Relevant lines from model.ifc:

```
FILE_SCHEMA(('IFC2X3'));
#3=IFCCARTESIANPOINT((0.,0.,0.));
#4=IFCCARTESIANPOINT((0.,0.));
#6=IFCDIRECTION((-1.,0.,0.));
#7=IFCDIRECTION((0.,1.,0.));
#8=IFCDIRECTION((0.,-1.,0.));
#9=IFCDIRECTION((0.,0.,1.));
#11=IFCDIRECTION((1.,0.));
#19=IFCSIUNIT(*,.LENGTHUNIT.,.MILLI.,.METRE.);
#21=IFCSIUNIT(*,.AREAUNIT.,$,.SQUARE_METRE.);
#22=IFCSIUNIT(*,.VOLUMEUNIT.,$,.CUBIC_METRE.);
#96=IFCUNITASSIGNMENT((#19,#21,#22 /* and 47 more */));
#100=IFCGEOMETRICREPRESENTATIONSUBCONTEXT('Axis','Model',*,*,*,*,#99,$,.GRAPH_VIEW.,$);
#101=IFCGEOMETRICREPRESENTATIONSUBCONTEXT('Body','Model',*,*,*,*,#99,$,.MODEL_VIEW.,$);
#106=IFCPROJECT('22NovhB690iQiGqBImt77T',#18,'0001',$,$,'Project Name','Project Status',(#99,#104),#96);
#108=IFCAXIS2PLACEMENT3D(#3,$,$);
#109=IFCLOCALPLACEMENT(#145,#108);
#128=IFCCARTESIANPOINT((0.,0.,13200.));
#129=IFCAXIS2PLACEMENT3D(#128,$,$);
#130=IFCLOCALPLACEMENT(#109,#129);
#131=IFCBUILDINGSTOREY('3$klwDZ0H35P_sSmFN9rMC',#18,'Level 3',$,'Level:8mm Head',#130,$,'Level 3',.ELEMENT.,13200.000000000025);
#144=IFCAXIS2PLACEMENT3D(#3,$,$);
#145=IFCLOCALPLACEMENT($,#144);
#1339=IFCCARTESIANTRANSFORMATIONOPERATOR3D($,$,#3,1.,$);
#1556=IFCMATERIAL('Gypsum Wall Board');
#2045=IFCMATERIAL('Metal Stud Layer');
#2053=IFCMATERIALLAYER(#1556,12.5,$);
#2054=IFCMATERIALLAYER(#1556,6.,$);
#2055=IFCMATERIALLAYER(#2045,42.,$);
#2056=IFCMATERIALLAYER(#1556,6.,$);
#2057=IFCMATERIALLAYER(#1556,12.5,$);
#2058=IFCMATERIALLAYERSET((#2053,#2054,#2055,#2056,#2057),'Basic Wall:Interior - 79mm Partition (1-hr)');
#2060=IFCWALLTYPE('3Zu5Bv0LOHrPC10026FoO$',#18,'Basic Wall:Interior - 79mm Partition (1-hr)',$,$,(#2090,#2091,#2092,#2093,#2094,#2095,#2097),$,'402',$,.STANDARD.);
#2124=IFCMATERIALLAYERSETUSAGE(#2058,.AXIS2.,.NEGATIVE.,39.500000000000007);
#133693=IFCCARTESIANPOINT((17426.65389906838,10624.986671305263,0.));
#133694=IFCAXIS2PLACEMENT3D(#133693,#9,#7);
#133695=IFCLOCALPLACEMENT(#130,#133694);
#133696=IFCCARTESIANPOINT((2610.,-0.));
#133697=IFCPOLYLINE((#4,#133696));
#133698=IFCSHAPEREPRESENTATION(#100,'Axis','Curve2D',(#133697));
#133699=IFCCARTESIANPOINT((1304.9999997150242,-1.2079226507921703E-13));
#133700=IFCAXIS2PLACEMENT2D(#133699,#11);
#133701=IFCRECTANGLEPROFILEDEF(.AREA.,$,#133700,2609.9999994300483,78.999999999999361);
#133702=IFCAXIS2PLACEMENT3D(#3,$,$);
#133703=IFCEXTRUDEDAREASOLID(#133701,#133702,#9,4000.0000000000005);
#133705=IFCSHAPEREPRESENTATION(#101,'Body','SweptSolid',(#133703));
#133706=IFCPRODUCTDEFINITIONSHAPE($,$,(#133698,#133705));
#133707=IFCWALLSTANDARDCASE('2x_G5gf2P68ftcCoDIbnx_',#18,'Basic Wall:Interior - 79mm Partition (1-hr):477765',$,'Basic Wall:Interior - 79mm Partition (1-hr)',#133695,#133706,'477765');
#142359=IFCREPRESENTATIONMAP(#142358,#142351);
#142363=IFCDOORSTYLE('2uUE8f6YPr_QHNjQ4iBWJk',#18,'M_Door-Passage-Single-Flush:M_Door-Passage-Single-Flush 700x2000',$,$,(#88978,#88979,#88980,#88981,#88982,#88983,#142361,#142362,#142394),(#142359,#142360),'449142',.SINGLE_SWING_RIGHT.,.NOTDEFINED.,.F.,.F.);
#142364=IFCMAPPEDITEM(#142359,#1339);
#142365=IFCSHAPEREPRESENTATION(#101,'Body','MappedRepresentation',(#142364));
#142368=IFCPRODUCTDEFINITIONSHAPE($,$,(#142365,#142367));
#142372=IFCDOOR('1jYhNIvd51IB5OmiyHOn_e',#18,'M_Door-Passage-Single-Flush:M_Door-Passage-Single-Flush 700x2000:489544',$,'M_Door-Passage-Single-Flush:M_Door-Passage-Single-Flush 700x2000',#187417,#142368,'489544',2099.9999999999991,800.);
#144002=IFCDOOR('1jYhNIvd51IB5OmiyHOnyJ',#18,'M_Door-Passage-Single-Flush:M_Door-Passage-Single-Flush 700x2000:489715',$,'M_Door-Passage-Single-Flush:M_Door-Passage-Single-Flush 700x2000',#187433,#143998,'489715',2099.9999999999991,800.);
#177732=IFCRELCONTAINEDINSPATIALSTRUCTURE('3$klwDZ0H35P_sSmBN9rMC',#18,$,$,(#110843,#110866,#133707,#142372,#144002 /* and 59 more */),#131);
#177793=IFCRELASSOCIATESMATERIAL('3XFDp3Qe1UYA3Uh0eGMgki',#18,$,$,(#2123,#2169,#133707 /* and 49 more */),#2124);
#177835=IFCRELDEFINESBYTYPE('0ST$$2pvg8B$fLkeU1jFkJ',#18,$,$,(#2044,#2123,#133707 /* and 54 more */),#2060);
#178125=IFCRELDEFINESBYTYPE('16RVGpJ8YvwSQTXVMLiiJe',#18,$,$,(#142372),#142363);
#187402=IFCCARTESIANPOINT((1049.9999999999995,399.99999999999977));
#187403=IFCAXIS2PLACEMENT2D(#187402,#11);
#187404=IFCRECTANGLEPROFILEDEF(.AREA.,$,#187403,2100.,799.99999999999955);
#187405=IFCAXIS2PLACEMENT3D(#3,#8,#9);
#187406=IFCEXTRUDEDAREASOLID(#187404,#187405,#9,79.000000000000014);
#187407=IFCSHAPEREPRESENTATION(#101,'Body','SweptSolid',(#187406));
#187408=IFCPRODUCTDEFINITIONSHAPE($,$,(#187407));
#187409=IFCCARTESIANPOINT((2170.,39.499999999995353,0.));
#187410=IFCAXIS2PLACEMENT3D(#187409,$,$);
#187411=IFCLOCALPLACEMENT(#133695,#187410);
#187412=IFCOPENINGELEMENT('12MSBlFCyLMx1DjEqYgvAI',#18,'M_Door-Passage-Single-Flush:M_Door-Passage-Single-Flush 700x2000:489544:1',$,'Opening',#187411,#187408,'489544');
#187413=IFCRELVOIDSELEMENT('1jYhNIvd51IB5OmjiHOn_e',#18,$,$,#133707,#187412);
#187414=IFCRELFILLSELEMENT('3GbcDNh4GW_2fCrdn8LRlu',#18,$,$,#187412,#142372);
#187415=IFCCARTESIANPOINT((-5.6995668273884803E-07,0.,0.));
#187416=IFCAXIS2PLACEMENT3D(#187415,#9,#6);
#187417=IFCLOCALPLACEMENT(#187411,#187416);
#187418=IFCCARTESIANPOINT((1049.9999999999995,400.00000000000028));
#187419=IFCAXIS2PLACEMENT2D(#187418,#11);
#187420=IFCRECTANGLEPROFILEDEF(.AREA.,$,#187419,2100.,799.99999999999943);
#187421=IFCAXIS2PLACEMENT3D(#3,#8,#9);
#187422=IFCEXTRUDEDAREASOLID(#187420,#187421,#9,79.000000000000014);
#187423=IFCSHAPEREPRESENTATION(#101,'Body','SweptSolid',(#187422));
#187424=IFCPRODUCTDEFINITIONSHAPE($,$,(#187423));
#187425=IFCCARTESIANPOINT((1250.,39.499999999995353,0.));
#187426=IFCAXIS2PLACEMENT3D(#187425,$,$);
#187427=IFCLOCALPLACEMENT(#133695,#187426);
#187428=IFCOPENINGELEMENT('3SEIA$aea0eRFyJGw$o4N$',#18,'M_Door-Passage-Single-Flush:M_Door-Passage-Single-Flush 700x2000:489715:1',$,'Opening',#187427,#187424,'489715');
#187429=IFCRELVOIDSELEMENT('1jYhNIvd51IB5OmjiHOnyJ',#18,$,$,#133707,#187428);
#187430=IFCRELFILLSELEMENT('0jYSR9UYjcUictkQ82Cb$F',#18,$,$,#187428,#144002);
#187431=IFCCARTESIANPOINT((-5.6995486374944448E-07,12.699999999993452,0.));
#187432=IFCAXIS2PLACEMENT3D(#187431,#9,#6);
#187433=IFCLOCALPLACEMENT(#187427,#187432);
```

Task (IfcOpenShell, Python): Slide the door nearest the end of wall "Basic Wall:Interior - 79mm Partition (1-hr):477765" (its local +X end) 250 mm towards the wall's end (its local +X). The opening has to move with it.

```python
import ifcopenshell
import ifcopenshell.api.geometry
import ifcopenshell.util.placement

model = ifcopenshell.open("model.ifc")

door = model.by_guid("1jYhNIvd51IB5OmiyHOn_e")
opening = door.FillsVoids[0].RelatingOpeningElement
wall = opening.VoidsElements[0].RelatingBuildingElement

wall_matrix = ifcopenshell.util.placement.get_local_placement(wall.ObjectPlacement)
shift = wall_matrix[:3, 0] * 250.0
before = ifcopenshell.util.placement.get_local_placement(door.ObjectPlacement)[:3, 3].copy()

# The door is placed relative to its opening, so it follows when the opening moves.
matrix = ifcopenshell.util.placement.get_local_placement(opening.ObjectPlacement)
matrix[:3, 3] += shift
ifcopenshell.api.geometry.edit_object_placement(
    model, product=opening, matrix=matrix, is_si=False, should_transform_children=True
)

after = ifcopenshell.util.placement.get_local_placement(door.ObjectPlacement)[:3, 3]
print("door moved by", (after - before).round(3) + 0.0)

model.write("model_rev.ifc")
```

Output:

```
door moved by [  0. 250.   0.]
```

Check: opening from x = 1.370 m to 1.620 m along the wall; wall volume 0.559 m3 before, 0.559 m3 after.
